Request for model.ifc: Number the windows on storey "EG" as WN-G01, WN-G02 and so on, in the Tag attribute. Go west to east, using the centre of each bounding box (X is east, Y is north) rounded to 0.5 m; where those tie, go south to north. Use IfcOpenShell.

First a look at what the model holds.

```python
import ifcopenshell
import ifcopenshell.util.element
import ifcopenshell.util.placement

model = ifcopenshell.open("model.ifc")
print(model.schema)
storey = next(s for s in model.by_type("IfcBuildingStorey") if s.Name == "EG")
windows = [e for e in ifcopenshell.util.element.get_decomposition(storey) if e.is_a("IfcWindow")]
for e in sorted(windows, key=lambda e: e.id()):
    origin = ifcopenshell.util.placement.get_local_placement(e.ObjectPlacement)[:3, 3]
    print(e.id(), e.Tag, e.Name, origin.round(2) + 0.0, sep=" | ")
```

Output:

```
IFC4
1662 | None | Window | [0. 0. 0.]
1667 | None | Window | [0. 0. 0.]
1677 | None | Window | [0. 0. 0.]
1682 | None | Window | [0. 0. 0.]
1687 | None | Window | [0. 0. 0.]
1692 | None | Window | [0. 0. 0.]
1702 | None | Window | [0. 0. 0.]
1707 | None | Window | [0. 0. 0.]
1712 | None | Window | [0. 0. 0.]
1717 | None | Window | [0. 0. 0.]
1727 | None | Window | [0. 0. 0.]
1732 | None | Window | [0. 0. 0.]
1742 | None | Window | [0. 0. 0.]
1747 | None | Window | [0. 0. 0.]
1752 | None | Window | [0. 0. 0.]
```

```python
import ifcopenshell
import ifcopenshell.geom
import ifcopenshell.util.element
import ifcopenshell.util.shape

model = ifcopenshell.open("model.ifc")
settings = ifcopenshell.geom.settings()
settings.set("use-world-coords", True)


def centre(element):
    shape = ifcopenshell.geom.create_shape(settings, element)
    return ifcopenshell.util.shape.get_bbox_centroid(shape.geometry)


storey = next(s for s in model.by_type("IfcBuildingStorey") if s.Name == "EG")
windows = [e for e in ifcopenshell.util.element.get_decomposition(storey) if e.is_a("IfcWindow")]

# Insertion points can sit at a corner or the storey origin, so sort by the geometry (in metres).
centres = {e: centre(e) for e in windows}
windows.sort(key=lambda e: (round(centres[e][0] / 0.5), centres[e][1]))

for i, e in enumerate(windows, start=1):
    number = f"WN-G{i:02d}"
    e.Tag = number
    print(e.id(), number)

model.write("model_updated.ifc")
```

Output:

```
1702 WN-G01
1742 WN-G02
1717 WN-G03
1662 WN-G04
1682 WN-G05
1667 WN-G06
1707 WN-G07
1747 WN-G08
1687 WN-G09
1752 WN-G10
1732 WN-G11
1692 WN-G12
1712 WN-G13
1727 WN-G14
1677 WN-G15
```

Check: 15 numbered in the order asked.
